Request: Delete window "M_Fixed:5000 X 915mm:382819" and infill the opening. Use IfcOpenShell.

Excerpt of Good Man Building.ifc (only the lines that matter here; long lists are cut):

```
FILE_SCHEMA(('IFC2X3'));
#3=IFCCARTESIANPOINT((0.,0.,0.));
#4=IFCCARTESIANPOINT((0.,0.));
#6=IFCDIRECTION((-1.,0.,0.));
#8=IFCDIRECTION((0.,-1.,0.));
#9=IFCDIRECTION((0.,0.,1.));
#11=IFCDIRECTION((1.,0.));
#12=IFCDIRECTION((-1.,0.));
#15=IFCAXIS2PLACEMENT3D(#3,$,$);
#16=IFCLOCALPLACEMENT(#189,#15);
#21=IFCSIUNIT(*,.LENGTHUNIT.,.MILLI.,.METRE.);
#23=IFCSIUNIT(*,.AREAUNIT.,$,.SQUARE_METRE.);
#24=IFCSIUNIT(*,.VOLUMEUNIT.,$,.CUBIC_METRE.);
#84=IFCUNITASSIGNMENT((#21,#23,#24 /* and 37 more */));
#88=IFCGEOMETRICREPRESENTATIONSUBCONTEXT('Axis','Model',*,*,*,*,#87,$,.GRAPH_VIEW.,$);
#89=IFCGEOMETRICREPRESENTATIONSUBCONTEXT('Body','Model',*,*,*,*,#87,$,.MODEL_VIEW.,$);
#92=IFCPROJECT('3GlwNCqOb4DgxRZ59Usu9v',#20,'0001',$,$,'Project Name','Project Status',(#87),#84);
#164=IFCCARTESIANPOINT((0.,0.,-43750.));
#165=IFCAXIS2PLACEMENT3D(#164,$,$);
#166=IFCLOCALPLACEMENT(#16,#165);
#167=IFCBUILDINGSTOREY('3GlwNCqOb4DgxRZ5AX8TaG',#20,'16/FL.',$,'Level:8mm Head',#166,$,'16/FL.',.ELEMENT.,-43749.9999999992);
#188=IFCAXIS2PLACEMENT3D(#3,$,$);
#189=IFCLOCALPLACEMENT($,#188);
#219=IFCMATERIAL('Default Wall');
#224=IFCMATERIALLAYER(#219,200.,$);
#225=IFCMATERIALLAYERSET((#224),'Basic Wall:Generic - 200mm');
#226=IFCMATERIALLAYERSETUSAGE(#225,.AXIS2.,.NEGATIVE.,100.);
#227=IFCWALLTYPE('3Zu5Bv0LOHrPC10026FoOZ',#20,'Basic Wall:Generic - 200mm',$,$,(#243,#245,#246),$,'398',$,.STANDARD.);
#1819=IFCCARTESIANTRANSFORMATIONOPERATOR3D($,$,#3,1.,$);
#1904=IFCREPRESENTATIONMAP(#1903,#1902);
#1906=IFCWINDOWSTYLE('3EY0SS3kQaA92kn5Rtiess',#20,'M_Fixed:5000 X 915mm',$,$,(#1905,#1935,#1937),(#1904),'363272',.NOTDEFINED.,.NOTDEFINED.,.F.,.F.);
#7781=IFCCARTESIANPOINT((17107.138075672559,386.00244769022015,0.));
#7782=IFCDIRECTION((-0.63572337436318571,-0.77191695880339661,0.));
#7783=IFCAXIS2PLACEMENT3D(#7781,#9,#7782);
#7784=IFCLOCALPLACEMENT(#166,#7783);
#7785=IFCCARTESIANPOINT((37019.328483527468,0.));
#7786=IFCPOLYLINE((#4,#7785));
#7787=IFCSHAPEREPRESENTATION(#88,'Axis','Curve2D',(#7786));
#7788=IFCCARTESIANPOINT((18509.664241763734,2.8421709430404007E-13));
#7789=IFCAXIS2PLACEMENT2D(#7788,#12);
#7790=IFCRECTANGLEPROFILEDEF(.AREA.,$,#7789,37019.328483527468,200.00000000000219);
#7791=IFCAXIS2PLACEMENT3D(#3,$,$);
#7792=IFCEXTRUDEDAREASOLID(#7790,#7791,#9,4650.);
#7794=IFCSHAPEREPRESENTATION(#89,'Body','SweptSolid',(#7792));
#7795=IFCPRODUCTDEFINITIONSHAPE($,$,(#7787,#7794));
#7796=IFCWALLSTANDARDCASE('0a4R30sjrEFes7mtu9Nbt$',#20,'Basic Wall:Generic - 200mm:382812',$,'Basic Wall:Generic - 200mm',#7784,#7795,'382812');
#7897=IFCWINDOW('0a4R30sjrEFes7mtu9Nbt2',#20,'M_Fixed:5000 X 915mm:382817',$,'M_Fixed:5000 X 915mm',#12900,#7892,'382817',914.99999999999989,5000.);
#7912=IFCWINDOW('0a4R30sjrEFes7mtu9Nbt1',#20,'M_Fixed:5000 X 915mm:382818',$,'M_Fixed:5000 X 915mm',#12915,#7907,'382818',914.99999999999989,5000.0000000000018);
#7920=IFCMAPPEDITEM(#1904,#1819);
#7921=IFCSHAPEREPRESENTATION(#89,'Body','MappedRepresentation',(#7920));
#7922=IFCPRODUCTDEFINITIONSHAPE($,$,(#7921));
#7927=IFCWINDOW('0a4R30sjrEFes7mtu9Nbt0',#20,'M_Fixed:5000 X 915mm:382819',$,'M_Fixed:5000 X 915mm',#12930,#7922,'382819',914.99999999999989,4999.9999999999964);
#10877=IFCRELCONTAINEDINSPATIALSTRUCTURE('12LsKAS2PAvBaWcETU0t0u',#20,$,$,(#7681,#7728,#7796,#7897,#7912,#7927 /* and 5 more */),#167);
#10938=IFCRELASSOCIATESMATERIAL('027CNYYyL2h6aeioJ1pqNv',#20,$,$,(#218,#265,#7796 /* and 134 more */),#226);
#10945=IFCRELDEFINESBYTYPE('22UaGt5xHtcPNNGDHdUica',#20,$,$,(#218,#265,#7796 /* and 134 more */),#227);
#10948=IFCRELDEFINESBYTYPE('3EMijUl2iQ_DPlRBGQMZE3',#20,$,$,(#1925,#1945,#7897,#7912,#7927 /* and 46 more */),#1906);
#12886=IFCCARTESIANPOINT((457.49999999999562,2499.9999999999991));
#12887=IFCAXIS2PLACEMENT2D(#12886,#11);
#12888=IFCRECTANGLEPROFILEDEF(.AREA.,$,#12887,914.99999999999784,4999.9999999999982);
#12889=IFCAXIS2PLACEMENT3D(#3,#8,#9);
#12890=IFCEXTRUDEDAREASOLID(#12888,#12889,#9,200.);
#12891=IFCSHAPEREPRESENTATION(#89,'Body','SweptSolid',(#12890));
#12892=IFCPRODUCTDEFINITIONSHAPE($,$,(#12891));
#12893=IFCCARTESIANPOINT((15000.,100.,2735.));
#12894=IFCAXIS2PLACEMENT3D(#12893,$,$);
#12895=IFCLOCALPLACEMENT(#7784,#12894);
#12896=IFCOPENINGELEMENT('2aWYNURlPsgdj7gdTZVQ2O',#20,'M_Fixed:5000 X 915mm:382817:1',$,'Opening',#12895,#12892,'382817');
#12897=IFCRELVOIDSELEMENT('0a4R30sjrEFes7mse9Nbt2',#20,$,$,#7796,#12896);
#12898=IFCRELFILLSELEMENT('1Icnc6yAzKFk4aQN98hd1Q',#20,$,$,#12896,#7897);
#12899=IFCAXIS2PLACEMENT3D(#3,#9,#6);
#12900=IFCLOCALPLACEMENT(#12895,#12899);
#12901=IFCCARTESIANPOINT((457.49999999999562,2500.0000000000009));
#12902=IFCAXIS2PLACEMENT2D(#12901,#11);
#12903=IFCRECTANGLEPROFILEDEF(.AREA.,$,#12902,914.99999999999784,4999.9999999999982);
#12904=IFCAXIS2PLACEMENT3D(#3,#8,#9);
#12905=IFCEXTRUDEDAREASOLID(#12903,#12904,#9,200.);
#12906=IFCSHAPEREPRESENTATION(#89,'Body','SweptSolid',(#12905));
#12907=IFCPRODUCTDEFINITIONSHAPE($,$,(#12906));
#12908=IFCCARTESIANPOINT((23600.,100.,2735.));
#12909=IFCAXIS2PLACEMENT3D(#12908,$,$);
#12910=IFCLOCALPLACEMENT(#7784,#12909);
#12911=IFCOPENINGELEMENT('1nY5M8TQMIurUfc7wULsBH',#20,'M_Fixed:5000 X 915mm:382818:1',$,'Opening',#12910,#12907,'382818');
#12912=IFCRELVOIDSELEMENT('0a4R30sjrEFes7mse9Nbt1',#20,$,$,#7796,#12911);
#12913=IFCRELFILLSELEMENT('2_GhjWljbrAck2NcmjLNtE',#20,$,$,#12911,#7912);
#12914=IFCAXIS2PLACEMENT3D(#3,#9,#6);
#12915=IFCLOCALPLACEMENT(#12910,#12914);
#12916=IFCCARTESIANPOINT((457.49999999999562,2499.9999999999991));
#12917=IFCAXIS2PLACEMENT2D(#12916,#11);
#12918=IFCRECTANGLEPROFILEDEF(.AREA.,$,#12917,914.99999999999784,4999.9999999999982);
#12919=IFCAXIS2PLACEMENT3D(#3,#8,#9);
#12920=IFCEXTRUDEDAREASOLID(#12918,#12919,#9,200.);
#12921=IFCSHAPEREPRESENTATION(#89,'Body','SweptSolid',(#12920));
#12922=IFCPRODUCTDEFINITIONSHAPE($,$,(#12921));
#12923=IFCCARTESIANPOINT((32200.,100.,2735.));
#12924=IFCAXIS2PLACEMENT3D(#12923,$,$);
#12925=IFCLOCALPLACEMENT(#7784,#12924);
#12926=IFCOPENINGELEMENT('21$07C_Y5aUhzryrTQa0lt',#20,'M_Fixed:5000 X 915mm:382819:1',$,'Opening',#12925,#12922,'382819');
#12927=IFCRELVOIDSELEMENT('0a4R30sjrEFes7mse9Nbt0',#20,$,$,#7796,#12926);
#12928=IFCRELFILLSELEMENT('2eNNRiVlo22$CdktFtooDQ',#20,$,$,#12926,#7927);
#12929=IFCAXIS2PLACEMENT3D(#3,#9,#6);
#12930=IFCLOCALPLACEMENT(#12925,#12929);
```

```python
import ifcopenshell
import ifcopenshell.api.feature
import ifcopenshell.api.root
import ifcopenshell.geom
import ifcopenshell.util.shape

model = ifcopenshell.open("Good Man Building.ifc")
settings = ifcopenshell.geom.settings()


def volume(element):
    """Net volume in cubic metres, openings subtracted."""
    shape = ifcopenshell.geom.create_shape(settings, element)
    return ifcopenshell.util.shape.get_volume(shape.geometry)


window = model.by_guid("0a4R30sjrEFes7mtu9Nbt0")
opening = window.FillsVoids[0].RelatingOpeningElement
wall = opening.VoidsElements[0].RelatingBuildingElement
before = volume(wall)

ifcopenshell.api.root.remove_product(model, product=window)
ifcopenshell.api.feature.remove_feature(model, feature=opening)

after = volume(wall)

print(f"wall volume {before:.3f} -> {after:.3f} m3")

model.write("Good Man Building_updated.ifc")
```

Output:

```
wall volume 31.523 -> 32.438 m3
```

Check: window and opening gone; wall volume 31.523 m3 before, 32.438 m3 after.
